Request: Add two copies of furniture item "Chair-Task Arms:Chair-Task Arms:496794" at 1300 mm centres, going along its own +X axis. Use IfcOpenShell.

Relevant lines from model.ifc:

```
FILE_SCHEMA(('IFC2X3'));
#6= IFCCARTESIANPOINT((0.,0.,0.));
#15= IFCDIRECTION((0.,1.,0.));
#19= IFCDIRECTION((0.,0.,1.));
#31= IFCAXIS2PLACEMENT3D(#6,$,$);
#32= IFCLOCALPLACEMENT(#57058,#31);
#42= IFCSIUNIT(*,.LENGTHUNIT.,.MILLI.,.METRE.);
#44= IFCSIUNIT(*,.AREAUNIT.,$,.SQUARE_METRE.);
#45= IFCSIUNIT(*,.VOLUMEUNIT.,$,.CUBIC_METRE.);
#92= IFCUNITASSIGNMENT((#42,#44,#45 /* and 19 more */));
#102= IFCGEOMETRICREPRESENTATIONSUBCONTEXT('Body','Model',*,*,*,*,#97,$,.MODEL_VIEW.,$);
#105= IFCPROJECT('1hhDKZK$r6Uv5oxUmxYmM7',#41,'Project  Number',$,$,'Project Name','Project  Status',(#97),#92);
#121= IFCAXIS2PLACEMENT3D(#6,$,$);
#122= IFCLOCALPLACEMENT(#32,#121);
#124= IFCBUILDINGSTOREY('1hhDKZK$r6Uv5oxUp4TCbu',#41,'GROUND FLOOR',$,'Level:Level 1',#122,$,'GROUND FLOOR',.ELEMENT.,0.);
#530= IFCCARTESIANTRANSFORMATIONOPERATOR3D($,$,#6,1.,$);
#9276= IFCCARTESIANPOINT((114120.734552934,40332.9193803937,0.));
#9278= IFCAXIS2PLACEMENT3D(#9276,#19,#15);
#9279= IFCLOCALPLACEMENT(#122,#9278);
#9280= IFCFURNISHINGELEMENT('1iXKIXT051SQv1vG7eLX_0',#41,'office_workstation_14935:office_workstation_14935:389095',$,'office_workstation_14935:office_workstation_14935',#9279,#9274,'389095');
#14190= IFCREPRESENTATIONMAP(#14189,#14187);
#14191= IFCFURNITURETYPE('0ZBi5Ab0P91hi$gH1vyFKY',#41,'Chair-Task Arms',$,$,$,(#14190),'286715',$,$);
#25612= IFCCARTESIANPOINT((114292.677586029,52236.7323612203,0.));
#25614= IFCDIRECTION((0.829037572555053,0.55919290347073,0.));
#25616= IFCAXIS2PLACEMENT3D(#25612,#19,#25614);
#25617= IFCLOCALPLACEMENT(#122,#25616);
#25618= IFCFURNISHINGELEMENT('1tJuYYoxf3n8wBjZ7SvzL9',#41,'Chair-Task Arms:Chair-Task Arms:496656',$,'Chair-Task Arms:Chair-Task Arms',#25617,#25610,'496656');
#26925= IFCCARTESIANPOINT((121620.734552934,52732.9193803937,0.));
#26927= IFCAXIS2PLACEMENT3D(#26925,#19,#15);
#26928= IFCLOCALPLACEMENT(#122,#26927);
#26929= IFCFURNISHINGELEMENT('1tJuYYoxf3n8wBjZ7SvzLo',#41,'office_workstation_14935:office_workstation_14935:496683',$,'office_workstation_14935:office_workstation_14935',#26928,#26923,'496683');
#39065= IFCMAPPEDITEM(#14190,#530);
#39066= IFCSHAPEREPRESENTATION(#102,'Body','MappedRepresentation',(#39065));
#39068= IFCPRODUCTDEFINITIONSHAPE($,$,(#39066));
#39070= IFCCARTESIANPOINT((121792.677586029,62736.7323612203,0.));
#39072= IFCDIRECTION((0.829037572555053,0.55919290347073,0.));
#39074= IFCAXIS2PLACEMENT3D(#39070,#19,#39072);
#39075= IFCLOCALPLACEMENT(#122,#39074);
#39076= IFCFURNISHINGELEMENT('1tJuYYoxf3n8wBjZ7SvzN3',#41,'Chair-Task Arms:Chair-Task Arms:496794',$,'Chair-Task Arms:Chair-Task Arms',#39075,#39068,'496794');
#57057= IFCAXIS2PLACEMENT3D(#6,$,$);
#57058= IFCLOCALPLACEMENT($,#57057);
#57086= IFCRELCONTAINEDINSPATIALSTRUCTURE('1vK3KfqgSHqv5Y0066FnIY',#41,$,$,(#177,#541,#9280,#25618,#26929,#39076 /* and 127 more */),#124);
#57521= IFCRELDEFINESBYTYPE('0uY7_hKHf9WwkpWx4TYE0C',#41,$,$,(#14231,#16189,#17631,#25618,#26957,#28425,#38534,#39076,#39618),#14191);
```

```python
import ifcopenshell
import ifcopenshell.api.geometry
import ifcopenshell.api.root
import ifcopenshell.util.element
import ifcopenshell.util.placement
import ifcopenshell.util.unit

model = ifcopenshell.open("model.ifc")
unit_scale = ifcopenshell.util.unit.calculate_unit_scale(model)


def reuse_history(source, copy):
    """copy_class also copies each property set's owner history, people and application; keep the originals."""
    for rel in copy.IsDefinedBy:
        if rel.is_a("IfcRelDefinesByProperties") and (history := rel.RelatingPropertyDefinition.OwnerHistory):
            rel.RelatingPropertyDefinition.OwnerHistory = source.OwnerHistory
            ifcopenshell.util.element.remove_deep2(model, history)


source = model.by_id(39076)
base = ifcopenshell.util.placement.get_local_placement(source.ObjectPlacement)
step = base[:3, 0] * 1.3 / unit_scale

for i in range(1, 3):
    copy = ifcopenshell.api.root.copy_class(model, product=source)
    copy.Representation = ifcopenshell.util.element.copy_deep(
        model, source.Representation, exclude=["IfcGeometricRepresentationContext", "IfcRepresentationMap"]
    )
    copy.Name = "Chair-Task Arms:Chair-Task Arms"
    copy.Tag = None
    reuse_history(source, copy)
    matrix = base.copy()
    matrix[:3, 3] += i * step
    print("added at", matrix[:3, 3].round(3) + 0.0)
    ifcopenshell.api.geometry.edit_object_placement(model, product=copy, matrix=matrix, is_si=False)

model.write("model_edited.ifc")
```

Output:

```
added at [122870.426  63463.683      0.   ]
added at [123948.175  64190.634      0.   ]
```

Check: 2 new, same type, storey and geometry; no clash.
